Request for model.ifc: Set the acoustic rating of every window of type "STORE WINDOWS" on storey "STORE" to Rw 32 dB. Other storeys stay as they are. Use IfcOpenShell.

First a look at what the model holds.

```python
import ifcopenshell
import ifcopenshell.util.element

model = ifcopenshell.open("model.ifc")
print(model.schema)
storey = next(s for s in model.by_type("IfcBuildingStorey") if s.Name == "STORE")
windows = [e for e in ifcopenshell.util.element.get_decomposition(storey) if e.is_a("IfcWindow")]
seen = {}
for e in windows:
    element_type = ifcopenshell.util.element.get_type(e)
    key = (element_type.Name if element_type != e and element_type else None, ifcopenshell.util.element.get_pset(e, "Pset_WindowCommon", "AcousticRating"))
    seen[key] = seen.get(key, 0) + 1
for (name, value), count in sorted(seen.items(), key=str):
    print(count, "x", name, "|", value)
```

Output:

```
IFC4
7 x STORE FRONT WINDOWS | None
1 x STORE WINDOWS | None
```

```python
import ifcopenshell
import ifcopenshell.api.pset
import ifcopenshell.util.element

model = ifcopenshell.open("model.ifc")

storey = next(s for s in model.by_type("IfcBuildingStorey") if s.Name == "STORE")
windows = [e for e in ifcopenshell.util.element.get_decomposition(storey) if e.is_a("IfcWindow")]

count = 0
for e in windows:
    element_type = ifcopenshell.util.element.get_type(e)
    if element_type in (None, e) or element_type.Name != "STORE WINDOWS":
        continue
    # add_pset returns the element's existing set when there is one.
    pset = ifcopenshell.api.pset.add_pset(model, product=e, name="Pset_WindowCommon")
    ifcopenshell.api.pset.edit_pset(model, pset=pset, properties={"AcousticRating": "Rw 32 dB"})
    count += 1

print(count, "windows updated")

model.write("model_v2.ifc")
```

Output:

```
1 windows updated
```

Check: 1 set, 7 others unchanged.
